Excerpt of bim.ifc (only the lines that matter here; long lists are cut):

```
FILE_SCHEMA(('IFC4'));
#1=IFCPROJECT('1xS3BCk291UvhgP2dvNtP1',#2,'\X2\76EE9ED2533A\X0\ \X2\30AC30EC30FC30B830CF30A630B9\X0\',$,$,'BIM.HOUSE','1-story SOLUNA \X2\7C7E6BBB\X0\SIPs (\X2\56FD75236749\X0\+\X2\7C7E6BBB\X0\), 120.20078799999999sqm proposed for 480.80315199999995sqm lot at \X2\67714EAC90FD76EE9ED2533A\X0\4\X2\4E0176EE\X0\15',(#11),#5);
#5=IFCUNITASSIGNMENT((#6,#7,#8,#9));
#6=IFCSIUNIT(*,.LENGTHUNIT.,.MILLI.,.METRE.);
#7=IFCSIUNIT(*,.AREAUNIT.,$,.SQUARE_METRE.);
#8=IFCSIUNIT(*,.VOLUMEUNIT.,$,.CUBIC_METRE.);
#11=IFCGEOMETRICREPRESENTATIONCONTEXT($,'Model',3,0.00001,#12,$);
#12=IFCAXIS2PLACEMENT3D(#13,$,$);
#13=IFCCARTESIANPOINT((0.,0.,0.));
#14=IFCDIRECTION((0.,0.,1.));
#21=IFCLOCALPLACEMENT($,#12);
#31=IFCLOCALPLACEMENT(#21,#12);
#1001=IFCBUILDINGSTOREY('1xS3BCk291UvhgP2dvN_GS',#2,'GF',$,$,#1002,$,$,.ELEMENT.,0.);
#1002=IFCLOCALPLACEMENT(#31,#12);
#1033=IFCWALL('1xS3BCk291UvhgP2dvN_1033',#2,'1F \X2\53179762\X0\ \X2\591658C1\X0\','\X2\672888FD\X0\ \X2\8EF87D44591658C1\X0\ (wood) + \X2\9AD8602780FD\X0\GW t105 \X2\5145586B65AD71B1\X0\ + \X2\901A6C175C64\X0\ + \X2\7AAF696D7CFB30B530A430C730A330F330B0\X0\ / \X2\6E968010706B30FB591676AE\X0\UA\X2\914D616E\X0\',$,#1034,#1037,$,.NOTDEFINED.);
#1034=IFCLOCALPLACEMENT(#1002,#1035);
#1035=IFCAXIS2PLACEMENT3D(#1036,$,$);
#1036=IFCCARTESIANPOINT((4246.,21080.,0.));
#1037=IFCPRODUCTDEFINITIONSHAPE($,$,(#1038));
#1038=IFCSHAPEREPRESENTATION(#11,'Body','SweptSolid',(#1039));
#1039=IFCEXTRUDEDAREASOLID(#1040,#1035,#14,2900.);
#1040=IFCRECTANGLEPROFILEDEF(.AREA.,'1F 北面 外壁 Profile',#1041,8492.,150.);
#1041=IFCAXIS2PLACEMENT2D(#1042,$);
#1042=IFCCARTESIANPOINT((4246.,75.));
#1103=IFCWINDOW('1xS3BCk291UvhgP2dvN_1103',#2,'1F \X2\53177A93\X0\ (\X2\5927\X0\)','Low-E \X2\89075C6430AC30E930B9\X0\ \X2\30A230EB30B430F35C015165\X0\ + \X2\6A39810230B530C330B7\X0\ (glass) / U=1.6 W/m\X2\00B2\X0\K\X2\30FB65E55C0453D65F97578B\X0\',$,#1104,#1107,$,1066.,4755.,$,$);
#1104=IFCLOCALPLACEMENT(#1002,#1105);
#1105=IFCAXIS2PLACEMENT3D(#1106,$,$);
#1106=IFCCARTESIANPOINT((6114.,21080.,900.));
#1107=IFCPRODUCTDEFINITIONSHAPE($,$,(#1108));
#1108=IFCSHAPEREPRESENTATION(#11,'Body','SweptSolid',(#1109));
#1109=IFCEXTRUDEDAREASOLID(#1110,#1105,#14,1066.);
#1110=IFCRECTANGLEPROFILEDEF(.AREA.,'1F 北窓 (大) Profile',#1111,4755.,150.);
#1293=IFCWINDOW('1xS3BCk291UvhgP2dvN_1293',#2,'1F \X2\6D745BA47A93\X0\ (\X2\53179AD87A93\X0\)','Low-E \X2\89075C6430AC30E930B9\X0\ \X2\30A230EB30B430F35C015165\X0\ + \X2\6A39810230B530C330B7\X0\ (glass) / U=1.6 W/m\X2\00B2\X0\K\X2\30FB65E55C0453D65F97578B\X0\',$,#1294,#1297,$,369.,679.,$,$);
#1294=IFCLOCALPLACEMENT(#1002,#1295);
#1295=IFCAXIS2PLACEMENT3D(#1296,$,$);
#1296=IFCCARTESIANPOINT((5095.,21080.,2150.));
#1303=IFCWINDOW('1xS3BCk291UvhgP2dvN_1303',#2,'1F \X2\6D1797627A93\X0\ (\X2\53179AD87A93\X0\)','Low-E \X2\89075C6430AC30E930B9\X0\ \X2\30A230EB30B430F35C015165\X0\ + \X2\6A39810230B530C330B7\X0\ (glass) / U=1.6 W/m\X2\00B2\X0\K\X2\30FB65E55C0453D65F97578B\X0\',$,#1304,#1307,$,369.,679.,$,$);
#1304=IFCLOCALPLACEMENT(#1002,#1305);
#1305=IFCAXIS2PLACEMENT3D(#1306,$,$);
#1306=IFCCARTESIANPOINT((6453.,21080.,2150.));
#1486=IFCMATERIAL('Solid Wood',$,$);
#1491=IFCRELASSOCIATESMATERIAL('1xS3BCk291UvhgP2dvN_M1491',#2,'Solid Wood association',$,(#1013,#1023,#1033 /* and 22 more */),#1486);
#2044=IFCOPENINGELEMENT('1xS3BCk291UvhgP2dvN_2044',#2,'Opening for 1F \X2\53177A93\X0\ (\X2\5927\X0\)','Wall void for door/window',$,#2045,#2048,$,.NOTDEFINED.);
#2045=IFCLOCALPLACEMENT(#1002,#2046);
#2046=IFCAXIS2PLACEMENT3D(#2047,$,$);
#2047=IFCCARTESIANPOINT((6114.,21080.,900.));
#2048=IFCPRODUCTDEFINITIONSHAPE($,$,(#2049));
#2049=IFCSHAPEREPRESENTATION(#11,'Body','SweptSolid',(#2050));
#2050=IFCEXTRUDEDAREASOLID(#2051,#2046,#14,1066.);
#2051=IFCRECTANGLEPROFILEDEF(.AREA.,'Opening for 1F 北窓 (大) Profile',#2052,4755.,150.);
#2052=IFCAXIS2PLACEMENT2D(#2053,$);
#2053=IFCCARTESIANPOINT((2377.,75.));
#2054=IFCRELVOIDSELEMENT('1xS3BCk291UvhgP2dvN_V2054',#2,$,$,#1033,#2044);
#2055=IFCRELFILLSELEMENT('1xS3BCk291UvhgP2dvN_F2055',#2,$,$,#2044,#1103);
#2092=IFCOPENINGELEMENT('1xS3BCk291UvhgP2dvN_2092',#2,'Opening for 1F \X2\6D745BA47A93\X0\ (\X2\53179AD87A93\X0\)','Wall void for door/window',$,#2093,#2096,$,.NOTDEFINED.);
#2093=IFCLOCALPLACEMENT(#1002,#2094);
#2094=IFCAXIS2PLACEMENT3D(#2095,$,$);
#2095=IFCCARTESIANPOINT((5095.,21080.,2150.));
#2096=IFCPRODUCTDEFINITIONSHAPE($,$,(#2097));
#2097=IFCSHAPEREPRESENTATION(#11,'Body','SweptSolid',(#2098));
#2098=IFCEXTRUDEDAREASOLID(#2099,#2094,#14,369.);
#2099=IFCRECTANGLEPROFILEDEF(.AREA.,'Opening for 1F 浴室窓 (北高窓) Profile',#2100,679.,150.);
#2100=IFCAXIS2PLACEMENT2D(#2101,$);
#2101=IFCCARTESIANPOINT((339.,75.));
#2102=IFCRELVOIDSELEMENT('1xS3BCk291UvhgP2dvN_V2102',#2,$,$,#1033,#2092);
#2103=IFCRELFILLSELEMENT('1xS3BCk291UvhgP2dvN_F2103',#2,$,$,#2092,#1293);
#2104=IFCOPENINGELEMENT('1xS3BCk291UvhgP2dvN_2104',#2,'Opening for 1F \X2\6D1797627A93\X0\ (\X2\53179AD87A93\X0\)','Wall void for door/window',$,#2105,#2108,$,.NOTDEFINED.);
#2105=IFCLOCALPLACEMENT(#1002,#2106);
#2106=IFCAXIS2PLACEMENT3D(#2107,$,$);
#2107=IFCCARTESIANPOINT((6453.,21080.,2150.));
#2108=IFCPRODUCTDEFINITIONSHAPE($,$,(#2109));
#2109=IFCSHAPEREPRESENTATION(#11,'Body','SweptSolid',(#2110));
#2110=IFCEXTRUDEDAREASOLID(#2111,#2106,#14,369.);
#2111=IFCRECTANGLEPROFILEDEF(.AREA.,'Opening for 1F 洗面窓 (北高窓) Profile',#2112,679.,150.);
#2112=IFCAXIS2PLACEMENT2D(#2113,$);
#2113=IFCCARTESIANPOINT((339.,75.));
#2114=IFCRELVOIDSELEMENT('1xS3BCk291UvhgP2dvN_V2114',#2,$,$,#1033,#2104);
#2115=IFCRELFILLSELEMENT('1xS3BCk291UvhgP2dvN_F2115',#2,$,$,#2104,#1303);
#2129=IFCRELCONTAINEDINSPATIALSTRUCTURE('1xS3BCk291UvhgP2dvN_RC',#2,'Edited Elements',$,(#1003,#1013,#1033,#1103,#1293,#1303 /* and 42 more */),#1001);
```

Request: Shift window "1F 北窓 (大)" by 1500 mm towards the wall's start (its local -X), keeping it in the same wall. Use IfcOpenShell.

```python
import ifcopenshell
import ifcopenshell.api.geometry
import ifcopenshell.util.placement
import ifcopenshell.util.unit

model = ifcopenshell.open("bim.ifc")
unit_scale = ifcopenshell.util.unit.calculate_unit_scale(model)

window = model.by_guid("1xS3BCk291UvhgP2dvN_1103")
opening = window.FillsVoids[0].RelatingOpeningElement
wall = opening.VoidsElements[0].RelatingBuildingElement

wall_matrix = ifcopenshell.util.placement.get_local_placement(wall.ObjectPlacement)
shift = wall_matrix[:3, 0] * -1.5 / unit_scale
before = ifcopenshell.util.placement.get_local_placement(window.ObjectPlacement)[:3, 3].copy()

# The window is not placed relative to its opening, so move both.
for product in (opening, window):
    matrix = ifcopenshell.util.placement.get_local_placement(product.ObjectPlacement)
    matrix[:3, 3] += shift
    ifcopenshell.api.geometry.edit_object_placement(model, product=product, matrix=matrix, is_si=False)

after = ifcopenshell.util.placement.get_local_placement(window.ObjectPlacement)[:3, 3]
print("window moved by", (after - before).round(3) + 0.0)

model.write("bim_updated.ifc")
```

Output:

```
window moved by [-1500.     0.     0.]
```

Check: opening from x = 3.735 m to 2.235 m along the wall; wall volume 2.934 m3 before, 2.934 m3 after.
